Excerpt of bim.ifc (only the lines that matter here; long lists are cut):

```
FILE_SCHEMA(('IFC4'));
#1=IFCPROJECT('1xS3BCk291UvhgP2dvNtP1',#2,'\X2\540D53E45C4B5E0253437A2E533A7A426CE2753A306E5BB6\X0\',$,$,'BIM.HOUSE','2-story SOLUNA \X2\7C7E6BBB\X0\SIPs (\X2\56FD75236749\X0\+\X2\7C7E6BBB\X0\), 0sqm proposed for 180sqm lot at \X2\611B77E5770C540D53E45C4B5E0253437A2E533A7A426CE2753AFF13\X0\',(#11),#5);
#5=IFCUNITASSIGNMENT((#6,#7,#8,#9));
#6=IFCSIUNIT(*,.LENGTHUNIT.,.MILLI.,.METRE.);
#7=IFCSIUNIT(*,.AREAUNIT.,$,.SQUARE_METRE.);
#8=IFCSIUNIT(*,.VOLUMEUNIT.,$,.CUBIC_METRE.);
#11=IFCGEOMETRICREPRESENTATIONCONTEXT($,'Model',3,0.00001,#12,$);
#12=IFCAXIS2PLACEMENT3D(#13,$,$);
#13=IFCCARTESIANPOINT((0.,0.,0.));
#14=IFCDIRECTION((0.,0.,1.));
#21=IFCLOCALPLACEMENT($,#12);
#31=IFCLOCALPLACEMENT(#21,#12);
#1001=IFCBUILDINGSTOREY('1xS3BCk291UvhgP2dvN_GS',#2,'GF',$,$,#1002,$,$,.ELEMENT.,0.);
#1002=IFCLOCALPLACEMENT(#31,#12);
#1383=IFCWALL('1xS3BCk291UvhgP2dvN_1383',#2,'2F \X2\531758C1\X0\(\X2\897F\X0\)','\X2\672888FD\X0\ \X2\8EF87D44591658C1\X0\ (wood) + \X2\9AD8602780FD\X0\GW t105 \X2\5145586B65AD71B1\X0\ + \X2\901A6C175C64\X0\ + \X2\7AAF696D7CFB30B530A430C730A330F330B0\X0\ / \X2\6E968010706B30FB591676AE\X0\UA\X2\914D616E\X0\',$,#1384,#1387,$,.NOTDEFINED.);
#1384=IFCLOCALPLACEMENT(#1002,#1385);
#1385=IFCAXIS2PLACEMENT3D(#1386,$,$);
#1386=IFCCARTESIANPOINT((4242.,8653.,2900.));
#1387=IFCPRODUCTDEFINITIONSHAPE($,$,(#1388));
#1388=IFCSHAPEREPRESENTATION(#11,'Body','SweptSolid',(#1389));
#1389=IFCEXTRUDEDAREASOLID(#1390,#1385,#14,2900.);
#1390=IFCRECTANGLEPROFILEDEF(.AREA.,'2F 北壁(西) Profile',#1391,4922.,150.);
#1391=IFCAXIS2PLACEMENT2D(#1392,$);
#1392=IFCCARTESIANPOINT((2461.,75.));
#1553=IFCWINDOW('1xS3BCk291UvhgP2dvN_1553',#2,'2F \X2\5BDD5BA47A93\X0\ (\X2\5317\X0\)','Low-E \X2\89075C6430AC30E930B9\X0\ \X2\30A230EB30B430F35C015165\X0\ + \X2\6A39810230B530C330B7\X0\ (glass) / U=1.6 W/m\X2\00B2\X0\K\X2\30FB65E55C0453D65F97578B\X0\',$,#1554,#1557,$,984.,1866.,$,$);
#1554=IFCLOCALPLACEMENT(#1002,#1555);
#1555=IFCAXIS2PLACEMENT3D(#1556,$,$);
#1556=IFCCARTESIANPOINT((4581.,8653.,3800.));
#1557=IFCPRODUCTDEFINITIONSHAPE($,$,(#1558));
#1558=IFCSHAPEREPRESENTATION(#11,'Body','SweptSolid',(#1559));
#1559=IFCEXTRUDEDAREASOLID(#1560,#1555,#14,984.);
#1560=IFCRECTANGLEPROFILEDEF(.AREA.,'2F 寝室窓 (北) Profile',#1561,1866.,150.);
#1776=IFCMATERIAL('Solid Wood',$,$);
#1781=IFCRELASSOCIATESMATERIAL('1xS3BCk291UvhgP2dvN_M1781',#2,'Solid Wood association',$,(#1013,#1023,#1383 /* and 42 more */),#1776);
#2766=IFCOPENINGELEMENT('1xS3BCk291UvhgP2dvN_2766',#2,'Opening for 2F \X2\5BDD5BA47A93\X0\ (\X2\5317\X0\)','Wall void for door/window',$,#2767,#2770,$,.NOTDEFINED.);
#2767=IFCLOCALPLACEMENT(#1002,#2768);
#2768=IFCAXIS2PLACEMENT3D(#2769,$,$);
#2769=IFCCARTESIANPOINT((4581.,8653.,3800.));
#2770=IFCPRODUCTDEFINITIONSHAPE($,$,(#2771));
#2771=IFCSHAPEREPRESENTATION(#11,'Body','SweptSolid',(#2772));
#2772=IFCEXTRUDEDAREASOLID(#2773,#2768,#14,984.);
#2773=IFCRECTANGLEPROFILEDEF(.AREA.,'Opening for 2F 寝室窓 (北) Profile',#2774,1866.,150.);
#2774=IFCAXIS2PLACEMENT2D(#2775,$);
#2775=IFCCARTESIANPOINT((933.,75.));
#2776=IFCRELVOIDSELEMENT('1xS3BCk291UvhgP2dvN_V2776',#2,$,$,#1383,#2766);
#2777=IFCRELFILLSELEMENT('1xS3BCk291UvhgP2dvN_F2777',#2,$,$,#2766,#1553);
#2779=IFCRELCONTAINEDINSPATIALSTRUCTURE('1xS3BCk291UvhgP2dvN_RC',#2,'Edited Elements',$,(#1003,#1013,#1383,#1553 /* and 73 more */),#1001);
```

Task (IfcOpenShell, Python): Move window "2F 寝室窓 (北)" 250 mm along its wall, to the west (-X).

```python
import ifcopenshell
import ifcopenshell.api.geometry
import ifcopenshell.util.placement
import ifcopenshell.util.unit

model = ifcopenshell.open("bim.ifc")
unit_scale = ifcopenshell.util.unit.calculate_unit_scale(model)

window = model.by_guid("1xS3BCk291UvhgP2dvN_1553")
opening = window.FillsVoids[0].RelatingOpeningElement
wall = opening.VoidsElements[0].RelatingBuildingElement

wall_matrix = ifcopenshell.util.placement.get_local_placement(wall.ObjectPlacement)
shift = wall_matrix[:3, 0] * -0.25 / unit_scale
before = ifcopenshell.util.placement.get_local_placement(window.ObjectPlacement)[:3, 3].copy()

# The window is not placed relative to its opening, so move both.
for product in (opening, window):
    matrix = ifcopenshell.util.placement.get_local_placement(product.ObjectPlacement)
    matrix[:3, 3] += shift
    ifcopenshell.api.geometry.edit_object_placement(model, product=product, matrix=matrix, is_si=False)

after = ifcopenshell.util.placement.get_local_placement(window.ObjectPlacement)[:3, 3]
print("window moved by", (after - before).round(3) + 0.0)

model.write("bim_rev.ifc")
```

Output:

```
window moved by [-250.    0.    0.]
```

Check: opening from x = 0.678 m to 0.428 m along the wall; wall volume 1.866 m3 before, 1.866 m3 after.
